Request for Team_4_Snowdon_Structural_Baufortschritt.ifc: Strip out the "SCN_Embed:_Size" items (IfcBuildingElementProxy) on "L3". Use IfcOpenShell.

First a look at what the model holds.

```python
import ifcopenshell
import ifcopenshell.util.element

model = ifcopenshell.open("Team_4_Snowdon_Structural_Baufortschritt.ifc")
print(model.schema)
storey = next(s for s in model.by_type("IfcBuildingStorey") if s.Name == "L3")
proxies = [e for e in ifcopenshell.util.element.get_decomposition(storey) if e.is_a("IfcBuildingElementProxy")]
seen = {}
for e in proxies:
    element_type = ifcopenshell.util.element.get_type(e)
    name = element_type.Name if element_type not in (None, e) else None
    seen[name] = seen.get(name, 0) + 1
for name, count in sorted(seen.items(), key=str):
    print(count, "x", name)
```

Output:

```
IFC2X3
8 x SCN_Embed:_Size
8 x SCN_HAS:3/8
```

```python
import ifcopenshell
import ifcopenshell.api.root
import ifcopenshell.util.element

model = ifcopenshell.open("Team_4_Snowdon_Structural_Baufortschritt.ifc")

storey = next(s for s in model.by_type("IfcBuildingStorey") if s.Name == "L3")
proxies = [e for e in ifcopenshell.util.element.get_decomposition(storey) if e.is_a("IfcBuildingElementProxy")]
targets = [e for e in proxies if (t := ifcopenshell.util.element.get_type(e)) not in (None, e) and t.Name == "SCN_Embed:_Size"]

for e in targets:
    ifcopenshell.api.root.remove_product(model, product=e)
print(len(targets), "removed")

model.write("Team_4_Snowdon_Structural_Baufortschritt_v2.ifc")
```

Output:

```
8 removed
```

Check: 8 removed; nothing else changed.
